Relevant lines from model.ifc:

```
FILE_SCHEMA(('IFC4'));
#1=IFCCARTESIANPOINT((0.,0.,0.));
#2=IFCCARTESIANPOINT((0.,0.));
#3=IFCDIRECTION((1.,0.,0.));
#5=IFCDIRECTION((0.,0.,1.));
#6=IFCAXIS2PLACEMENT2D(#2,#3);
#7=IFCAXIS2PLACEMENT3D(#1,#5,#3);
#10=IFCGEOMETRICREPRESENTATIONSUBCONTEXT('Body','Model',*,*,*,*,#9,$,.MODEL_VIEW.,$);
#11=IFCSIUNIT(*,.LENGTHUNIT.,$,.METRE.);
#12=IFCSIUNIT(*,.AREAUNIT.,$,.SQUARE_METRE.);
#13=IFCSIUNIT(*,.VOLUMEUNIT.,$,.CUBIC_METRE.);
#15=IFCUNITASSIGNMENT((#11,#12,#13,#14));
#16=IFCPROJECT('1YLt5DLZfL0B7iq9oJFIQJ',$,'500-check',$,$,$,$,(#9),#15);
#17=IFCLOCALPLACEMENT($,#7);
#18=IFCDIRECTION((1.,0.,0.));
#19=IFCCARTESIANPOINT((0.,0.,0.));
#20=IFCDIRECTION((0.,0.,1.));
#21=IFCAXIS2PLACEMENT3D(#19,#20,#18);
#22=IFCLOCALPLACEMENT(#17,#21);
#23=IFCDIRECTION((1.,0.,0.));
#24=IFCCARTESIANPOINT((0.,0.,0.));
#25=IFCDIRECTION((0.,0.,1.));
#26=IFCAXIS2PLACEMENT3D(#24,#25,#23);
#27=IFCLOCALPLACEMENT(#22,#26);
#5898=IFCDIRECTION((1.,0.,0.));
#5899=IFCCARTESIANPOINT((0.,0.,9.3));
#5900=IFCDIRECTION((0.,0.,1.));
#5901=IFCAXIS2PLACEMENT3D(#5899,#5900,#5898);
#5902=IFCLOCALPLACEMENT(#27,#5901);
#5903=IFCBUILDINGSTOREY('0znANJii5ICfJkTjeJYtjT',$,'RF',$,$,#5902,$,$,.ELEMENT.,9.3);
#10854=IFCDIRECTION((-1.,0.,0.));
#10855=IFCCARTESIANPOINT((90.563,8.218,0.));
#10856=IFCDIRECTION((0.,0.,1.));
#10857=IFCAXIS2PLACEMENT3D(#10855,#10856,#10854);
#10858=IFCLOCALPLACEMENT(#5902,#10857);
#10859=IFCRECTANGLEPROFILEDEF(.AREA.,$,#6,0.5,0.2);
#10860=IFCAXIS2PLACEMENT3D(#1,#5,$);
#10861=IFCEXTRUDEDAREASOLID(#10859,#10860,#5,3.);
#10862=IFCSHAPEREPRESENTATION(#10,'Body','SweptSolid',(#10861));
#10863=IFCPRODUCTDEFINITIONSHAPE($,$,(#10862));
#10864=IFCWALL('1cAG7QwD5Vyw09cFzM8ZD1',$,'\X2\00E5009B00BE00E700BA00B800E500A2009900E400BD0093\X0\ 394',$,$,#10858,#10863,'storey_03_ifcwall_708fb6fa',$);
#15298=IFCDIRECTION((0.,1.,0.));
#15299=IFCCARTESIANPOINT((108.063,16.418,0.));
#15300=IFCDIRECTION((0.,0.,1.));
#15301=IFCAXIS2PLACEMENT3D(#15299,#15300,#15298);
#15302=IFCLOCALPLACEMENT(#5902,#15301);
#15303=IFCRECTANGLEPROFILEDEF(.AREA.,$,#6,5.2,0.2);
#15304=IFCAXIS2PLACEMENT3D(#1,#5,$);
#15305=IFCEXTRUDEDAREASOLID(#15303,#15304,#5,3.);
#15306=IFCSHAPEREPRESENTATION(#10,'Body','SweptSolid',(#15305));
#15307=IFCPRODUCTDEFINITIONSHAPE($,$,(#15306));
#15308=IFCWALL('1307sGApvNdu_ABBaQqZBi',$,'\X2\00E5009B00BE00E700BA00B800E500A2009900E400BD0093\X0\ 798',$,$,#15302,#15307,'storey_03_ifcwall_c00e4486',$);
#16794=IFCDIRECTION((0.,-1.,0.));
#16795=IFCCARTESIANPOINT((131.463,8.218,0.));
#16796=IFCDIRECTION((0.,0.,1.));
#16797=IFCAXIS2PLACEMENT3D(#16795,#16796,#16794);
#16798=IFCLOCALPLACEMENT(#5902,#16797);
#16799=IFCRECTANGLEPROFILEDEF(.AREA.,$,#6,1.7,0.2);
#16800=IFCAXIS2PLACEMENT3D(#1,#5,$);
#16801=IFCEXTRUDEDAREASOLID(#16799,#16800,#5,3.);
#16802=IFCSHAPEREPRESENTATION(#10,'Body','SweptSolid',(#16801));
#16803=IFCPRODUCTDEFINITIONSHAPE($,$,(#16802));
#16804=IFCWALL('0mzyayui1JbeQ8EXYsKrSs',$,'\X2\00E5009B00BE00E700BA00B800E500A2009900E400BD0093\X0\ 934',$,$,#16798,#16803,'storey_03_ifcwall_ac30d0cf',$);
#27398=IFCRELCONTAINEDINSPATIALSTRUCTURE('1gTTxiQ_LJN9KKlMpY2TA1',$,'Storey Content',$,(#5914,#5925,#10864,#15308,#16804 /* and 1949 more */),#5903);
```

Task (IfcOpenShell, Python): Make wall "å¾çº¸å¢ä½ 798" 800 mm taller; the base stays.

```python
import ifcopenshell
import ifcopenshell.geom
import ifcopenshell.util.representation
import ifcopenshell.util.shape
import ifcopenshell.util.unit

model = ifcopenshell.open("model.ifc")
unit_scale = ifcopenshell.util.unit.calculate_unit_scale(model)
settings = ifcopenshell.geom.settings()


def volume(element):
    """Net volume in cubic metres, openings subtracted."""
    shape = ifcopenshell.geom.create_shape(settings, element)
    return ifcopenshell.util.shape.get_volume(shape.geometry)


wall = model.by_guid("1307sGApvNdu_ABBaQqZBi")
before = volume(wall)

body = ifcopenshell.util.representation.get_representation(wall, "Model", "Body")
solid = body.Items[0]
old_height = solid.Depth
solid.Depth += 0.8 / unit_scale
after = volume(wall)

print(f"height {old_height:g} -> {solid.Depth:g}, volume {before:.3f} -> {after:.3f} m3")

model.write("model-out.ifc")
```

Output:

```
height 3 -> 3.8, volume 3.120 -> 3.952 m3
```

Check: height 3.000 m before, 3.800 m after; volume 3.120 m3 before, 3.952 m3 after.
